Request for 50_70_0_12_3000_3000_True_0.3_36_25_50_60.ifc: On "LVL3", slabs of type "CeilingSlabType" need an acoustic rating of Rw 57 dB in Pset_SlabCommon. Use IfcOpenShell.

First a look at what the model holds.

```python
import ifcopenshell
import ifcopenshell.util.element

model = ifcopenshell.open("50_70_0_12_3000_3000_True_0.3_36_25_50_60.ifc")
print(model.schema)
storey = next(s for s in model.by_type("IfcBuildingStorey") if s.Name == "LVL3")
slabs = [e for e in ifcopenshell.util.element.get_decomposition(storey) if e.is_a("IfcSlab")]
seen = {}
for e in slabs:
    element_type = ifcopenshell.util.element.get_type(e)
    key = (element_type.Name if element_type != e and element_type else None, ifcopenshell.util.element.get_pset(e, "Pset_SlabCommon", "AcousticRating"))
    seen[key] = seen.get(key, 0) + 1
for (name, value), count in sorted(seen.items(), key=str):
    print(count, "x", name, "|", value)
```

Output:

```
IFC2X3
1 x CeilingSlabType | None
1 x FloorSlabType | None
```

```python
import ifcopenshell
import ifcopenshell.api.pset
import ifcopenshell.util.element

model = ifcopenshell.open("50_70_0_12_3000_3000_True_0.3_36_25_50_60.ifc")

storey = next(s for s in model.by_type("IfcBuildingStorey") if s.Name == "LVL3")
slabs = [e for e in ifcopenshell.util.element.get_decomposition(storey) if e.is_a("IfcSlab")]

count = 0
for e in slabs:
    element_type = ifcopenshell.util.element.get_type(e)
    if element_type in (None, e) or element_type.Name != "CeilingSlabType":
        continue
    # add_pset returns the element's existing set when there is one.
    pset = ifcopenshell.api.pset.add_pset(model, product=e, name="Pset_SlabCommon")
    ifcopenshell.api.pset.edit_pset(model, pset=pset, properties={"AcousticRating": "Rw 57 dB"})
    count += 1

print(count, "slabs updated")

model.write("50_70_0_12_3000_3000_True_0.3_36_25_50_60_edited.ifc")
```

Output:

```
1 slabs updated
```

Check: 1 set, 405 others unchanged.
